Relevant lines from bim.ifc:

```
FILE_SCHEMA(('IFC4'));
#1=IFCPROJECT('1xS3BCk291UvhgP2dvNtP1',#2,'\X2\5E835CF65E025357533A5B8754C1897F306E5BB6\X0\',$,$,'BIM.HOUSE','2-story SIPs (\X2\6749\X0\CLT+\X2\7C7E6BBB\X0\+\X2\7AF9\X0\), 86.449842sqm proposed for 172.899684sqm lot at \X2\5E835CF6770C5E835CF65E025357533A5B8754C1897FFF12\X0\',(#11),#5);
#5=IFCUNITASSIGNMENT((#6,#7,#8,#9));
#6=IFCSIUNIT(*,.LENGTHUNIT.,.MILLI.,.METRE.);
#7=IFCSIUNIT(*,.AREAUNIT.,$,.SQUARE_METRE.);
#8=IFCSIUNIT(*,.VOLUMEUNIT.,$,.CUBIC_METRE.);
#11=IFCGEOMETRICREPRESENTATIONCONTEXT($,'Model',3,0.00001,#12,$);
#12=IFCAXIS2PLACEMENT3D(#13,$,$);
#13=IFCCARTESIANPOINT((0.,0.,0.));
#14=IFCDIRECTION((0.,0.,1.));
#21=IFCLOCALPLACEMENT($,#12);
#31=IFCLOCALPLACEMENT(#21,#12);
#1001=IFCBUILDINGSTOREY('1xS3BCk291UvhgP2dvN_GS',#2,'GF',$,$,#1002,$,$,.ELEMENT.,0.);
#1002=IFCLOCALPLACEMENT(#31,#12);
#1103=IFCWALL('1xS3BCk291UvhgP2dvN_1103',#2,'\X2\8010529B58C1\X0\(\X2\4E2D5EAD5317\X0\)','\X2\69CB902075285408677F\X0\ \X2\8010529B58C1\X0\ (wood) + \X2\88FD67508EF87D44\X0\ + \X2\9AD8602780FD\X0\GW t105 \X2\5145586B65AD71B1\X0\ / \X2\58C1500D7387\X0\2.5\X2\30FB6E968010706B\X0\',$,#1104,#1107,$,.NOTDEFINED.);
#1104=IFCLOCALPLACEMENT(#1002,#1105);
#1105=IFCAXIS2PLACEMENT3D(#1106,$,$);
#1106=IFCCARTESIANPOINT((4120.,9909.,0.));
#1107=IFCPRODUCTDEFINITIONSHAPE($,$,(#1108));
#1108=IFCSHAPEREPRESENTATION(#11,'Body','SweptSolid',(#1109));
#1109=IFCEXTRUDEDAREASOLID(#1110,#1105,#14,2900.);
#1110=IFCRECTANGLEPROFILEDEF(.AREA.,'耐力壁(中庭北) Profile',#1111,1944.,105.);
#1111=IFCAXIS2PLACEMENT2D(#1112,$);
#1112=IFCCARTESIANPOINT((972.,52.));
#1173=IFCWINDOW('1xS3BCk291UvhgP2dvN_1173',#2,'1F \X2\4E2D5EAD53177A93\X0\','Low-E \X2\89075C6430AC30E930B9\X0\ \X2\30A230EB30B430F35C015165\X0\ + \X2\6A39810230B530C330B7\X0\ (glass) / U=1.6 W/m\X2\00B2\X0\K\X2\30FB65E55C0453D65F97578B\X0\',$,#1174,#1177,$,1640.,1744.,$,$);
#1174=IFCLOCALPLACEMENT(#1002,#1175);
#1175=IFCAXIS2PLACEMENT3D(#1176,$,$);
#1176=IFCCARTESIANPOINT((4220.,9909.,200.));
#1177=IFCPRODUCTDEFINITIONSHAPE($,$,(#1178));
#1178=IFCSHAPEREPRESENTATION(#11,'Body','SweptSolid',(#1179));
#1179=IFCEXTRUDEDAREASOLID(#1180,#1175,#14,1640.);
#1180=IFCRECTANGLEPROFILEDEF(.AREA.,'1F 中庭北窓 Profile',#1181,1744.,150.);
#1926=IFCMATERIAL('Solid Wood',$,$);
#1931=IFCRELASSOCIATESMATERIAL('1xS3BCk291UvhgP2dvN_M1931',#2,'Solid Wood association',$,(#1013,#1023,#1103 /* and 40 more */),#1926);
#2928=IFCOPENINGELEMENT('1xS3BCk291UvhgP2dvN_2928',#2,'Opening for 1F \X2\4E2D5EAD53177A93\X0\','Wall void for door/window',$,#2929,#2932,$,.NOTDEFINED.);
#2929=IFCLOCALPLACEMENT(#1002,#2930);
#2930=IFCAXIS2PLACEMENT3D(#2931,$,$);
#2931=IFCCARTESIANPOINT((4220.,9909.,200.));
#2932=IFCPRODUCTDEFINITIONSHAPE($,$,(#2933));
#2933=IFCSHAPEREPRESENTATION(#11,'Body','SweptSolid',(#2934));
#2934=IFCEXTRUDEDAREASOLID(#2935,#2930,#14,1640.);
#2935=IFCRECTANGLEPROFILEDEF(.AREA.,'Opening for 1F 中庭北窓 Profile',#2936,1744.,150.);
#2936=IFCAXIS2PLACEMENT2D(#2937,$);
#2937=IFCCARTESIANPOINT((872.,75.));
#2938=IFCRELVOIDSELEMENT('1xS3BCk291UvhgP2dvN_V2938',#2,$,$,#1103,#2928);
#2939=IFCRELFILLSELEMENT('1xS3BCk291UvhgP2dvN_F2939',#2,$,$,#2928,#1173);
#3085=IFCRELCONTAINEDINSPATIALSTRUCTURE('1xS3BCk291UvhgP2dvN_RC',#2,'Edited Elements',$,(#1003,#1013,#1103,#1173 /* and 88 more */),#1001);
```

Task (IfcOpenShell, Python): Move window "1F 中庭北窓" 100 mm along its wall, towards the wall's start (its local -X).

```python
import ifcopenshell
import ifcopenshell.api.geometry
import ifcopenshell.util.placement
import ifcopenshell.util.unit

model = ifcopenshell.open("bim.ifc")
unit_scale = ifcopenshell.util.unit.calculate_unit_scale(model)

window = model.by_guid("1xS3BCk291UvhgP2dvN_1173")
opening = window.FillsVoids[0].RelatingOpeningElement
wall = opening.VoidsElements[0].RelatingBuildingElement

wall_matrix = ifcopenshell.util.placement.get_local_placement(wall.ObjectPlacement)
shift = wall_matrix[:3, 0] * -0.1 / unit_scale
before = ifcopenshell.util.placement.get_local_placement(window.ObjectPlacement)[:3, 3].copy()

# The window is not placed relative to its opening, so move both.
for product in (opening, window):
    matrix = ifcopenshell.util.placement.get_local_placement(product.ObjectPlacement)
    matrix[:3, 3] += shift
    ifcopenshell.api.geometry.edit_object_placement(model, product=product, matrix=matrix, is_si=False)

after = ifcopenshell.util.placement.get_local_placement(window.ObjectPlacement)[:3, 3]
print("window moved by", (after - before).round(3) + 0.0)

model.write("bim_edited.ifc")
```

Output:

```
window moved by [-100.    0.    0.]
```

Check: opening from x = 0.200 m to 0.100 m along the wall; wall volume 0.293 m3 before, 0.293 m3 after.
